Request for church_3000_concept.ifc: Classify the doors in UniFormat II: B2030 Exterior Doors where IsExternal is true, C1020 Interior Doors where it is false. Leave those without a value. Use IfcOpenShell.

First a look at what the model holds.

```python
import ifcopenshell
import ifcopenshell.util.element

model = ifcopenshell.open("church_3000_concept.ifc")
print(model.schema)
print("classifications:", [c.Name for c in model.by_type("IfcClassification")])
values = [ifcopenshell.util.element.get_pset(e, "Pset_DoorCommon", "IsExternal") for e in model.by_type("IfcDoor")]
for value in (True, False, None):
    print("IsExternal", value, values.count(value))
```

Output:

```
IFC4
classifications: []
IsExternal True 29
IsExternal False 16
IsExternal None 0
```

```python
import ifcopenshell
import ifcopenshell.api.classification
import ifcopenshell.util.element

model = ifcopenshell.open("church_3000_concept.ifc")

system = ifcopenshell.api.classification.add_classification(model, classification="UniFormat II")

doors = model.by_type("IfcDoor")
external = {e: ifcopenshell.util.element.get_pset(e, "Pset_DoorCommon", "IsExternal") for e in doors}
for flag, code, name in ((True, "B2030", "Exterior Doors"), (False, "C1020", "Interior Doors")):
    products = [e for e in doors if external[e] is flag]
    ifcopenshell.api.classification.add_reference(
        model, products=products, classification=system, identification=code, name=name
    )
    print(code, len(products))

model.write("church_3000_concept_v2.ifc")
```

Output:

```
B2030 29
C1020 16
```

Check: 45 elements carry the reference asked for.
